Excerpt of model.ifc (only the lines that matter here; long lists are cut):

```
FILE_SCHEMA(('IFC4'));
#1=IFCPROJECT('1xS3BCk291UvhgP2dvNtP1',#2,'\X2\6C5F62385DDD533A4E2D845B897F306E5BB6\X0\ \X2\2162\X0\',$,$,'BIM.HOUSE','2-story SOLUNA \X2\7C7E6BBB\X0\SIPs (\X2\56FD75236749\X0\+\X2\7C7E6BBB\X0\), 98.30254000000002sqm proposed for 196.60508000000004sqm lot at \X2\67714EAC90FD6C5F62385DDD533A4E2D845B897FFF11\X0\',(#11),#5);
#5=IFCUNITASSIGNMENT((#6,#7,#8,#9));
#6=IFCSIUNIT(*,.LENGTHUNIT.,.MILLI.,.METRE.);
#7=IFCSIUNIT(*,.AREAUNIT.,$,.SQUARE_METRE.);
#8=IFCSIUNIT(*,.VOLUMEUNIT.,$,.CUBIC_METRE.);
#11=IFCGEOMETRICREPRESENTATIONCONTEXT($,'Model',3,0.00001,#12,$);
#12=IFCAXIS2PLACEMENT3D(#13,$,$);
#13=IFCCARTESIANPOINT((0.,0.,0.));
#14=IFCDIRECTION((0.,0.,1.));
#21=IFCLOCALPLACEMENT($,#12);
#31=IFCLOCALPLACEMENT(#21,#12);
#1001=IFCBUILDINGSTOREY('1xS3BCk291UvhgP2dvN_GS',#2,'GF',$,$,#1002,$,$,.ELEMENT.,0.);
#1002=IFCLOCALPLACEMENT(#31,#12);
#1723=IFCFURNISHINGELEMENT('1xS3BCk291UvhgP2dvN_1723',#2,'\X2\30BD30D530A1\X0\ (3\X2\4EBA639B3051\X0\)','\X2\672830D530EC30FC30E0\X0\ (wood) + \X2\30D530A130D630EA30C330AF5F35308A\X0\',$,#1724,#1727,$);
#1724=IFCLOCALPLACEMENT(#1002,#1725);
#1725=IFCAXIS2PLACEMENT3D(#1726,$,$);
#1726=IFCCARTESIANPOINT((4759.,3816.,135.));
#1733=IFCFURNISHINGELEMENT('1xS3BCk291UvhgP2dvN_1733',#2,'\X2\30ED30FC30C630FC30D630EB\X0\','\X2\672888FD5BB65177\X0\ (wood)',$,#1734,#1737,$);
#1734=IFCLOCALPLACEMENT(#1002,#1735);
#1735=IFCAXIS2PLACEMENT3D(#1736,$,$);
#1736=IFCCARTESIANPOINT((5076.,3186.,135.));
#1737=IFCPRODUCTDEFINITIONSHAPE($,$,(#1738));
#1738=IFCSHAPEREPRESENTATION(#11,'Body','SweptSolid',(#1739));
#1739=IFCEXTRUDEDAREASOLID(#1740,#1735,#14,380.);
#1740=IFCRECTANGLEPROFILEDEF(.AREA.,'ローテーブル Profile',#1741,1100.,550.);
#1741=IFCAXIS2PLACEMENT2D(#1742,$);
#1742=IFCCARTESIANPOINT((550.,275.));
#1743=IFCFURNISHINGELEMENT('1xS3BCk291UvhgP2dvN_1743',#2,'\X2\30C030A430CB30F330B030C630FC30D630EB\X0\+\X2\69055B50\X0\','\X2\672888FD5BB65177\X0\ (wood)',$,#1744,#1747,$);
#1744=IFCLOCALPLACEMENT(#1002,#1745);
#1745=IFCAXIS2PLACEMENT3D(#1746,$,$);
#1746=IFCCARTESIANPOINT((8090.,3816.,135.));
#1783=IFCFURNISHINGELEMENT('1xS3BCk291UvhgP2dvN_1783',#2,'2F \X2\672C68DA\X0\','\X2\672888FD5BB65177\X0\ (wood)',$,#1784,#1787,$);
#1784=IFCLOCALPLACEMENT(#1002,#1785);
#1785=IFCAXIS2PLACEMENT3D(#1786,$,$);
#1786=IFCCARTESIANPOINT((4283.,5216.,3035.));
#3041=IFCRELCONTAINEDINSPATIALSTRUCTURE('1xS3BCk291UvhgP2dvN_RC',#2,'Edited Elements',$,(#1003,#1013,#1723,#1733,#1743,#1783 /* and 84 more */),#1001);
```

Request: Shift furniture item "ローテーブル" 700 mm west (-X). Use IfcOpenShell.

```python
import ifcopenshell
import ifcopenshell.api.geometry
import ifcopenshell.util.placement
import ifcopenshell.util.unit

model = ifcopenshell.open("model.ifc")
unit_scale = ifcopenshell.util.unit.calculate_unit_scale(model)

item = model.by_guid("1xS3BCk291UvhgP2dvN_1733")
matrix = ifcopenshell.util.placement.get_local_placement(item.ObjectPlacement)
matrix[0, 3] -= 0.7 / unit_scale
ifcopenshell.api.geometry.edit_object_placement(model, product=item, matrix=matrix, is_si=False)

print(ifcopenshell.util.placement.get_local_placement(item.ObjectPlacement).round(3) + 0.0)

model.write("model_updated.ifc")
```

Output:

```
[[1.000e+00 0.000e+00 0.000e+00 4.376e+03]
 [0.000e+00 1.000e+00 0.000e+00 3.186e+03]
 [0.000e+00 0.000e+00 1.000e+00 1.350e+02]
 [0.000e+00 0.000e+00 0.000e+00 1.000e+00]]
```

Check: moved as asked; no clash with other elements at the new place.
